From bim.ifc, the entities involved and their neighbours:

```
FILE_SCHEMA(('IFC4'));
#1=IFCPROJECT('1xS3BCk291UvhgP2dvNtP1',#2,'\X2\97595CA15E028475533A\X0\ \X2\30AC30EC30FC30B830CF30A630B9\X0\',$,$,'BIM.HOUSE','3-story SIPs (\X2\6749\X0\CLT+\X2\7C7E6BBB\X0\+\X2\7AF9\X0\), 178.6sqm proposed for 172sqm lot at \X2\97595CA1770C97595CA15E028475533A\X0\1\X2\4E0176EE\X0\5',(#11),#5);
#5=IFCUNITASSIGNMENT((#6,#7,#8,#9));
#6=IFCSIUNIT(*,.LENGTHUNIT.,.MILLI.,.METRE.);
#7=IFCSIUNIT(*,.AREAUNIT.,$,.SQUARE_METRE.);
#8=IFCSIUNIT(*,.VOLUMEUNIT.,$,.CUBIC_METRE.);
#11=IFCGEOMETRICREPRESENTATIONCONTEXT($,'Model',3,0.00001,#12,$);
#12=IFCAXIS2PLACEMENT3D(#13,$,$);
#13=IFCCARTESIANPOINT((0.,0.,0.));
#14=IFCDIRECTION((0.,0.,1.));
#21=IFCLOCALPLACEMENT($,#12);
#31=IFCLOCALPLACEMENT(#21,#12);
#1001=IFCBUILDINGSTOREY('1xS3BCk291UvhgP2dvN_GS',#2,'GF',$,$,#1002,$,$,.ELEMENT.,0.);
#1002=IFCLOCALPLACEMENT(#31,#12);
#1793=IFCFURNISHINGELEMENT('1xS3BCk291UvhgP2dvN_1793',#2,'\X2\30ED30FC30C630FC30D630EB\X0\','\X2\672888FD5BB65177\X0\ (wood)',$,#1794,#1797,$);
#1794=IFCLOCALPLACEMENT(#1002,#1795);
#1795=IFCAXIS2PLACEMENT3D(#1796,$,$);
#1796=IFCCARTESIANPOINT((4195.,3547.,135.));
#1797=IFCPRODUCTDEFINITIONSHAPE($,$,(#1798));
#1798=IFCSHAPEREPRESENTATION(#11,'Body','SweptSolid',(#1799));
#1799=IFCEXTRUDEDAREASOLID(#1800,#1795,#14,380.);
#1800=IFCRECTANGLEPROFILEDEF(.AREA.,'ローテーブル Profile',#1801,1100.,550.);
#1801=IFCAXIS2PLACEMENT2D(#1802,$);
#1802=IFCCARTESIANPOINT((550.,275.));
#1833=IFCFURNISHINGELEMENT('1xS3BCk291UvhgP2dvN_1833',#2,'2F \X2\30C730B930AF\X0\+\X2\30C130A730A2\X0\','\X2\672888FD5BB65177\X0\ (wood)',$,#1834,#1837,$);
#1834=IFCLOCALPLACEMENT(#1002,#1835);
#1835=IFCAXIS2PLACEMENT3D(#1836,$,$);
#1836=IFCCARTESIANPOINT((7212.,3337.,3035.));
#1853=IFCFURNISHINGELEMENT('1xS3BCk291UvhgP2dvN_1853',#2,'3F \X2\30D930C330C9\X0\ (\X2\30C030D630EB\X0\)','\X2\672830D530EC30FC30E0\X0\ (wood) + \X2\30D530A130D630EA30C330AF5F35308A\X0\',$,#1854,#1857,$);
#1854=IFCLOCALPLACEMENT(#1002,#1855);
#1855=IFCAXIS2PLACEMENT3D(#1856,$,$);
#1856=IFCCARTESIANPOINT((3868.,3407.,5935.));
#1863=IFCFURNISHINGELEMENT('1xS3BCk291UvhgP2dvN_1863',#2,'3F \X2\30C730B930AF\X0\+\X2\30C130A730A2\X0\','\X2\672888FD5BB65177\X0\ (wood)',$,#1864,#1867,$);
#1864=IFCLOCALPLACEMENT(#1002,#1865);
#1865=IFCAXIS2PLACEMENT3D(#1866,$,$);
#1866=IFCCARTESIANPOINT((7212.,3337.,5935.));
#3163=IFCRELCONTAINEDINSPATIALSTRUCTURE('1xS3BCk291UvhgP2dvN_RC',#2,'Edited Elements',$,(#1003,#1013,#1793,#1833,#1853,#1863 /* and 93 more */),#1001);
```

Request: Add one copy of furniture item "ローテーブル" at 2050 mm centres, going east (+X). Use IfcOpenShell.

```python
import numpy as np
import ifcopenshell
import ifcopenshell.api.geometry
import ifcopenshell.api.root
import ifcopenshell.util.element
import ifcopenshell.util.placement
import ifcopenshell.util.unit

model = ifcopenshell.open("bim.ifc")
unit_scale = ifcopenshell.util.unit.calculate_unit_scale(model)


def reuse_history(source, copy):
    """copy_class also copies each property set's owner history, people and application; keep the originals."""
    for rel in copy.IsDefinedBy:
        if rel.is_a("IfcRelDefinesByProperties") and (history := rel.RelatingPropertyDefinition.OwnerHistory):
            rel.RelatingPropertyDefinition.OwnerHistory = source.OwnerHistory
            ifcopenshell.util.element.remove_deep2(model, history)


source = model.by_guid("1xS3BCk291UvhgP2dvN_1793")
base = ifcopenshell.util.placement.get_local_placement(source.ObjectPlacement)
step = np.array([1.0, 0.0, 0.0]) * 2.05 / unit_scale

for i in range(1, 2):
    copy = ifcopenshell.api.root.copy_class(model, product=source)
    copy.Representation = ifcopenshell.util.element.copy_deep(
        model, source.Representation, exclude=["IfcGeometricRepresentationContext", "IfcRepresentationMap"]
    )
    reuse_history(source, copy)
    matrix = base.copy()
    matrix[:3, 3] += i * step
    print("added at", matrix[:3, 3].round(3) + 0.0)
    ifcopenshell.api.geometry.edit_object_placement(model, product=copy, matrix=matrix, is_si=False)

model.write("bim_v2.ifc")
```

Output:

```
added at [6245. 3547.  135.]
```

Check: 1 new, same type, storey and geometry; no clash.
